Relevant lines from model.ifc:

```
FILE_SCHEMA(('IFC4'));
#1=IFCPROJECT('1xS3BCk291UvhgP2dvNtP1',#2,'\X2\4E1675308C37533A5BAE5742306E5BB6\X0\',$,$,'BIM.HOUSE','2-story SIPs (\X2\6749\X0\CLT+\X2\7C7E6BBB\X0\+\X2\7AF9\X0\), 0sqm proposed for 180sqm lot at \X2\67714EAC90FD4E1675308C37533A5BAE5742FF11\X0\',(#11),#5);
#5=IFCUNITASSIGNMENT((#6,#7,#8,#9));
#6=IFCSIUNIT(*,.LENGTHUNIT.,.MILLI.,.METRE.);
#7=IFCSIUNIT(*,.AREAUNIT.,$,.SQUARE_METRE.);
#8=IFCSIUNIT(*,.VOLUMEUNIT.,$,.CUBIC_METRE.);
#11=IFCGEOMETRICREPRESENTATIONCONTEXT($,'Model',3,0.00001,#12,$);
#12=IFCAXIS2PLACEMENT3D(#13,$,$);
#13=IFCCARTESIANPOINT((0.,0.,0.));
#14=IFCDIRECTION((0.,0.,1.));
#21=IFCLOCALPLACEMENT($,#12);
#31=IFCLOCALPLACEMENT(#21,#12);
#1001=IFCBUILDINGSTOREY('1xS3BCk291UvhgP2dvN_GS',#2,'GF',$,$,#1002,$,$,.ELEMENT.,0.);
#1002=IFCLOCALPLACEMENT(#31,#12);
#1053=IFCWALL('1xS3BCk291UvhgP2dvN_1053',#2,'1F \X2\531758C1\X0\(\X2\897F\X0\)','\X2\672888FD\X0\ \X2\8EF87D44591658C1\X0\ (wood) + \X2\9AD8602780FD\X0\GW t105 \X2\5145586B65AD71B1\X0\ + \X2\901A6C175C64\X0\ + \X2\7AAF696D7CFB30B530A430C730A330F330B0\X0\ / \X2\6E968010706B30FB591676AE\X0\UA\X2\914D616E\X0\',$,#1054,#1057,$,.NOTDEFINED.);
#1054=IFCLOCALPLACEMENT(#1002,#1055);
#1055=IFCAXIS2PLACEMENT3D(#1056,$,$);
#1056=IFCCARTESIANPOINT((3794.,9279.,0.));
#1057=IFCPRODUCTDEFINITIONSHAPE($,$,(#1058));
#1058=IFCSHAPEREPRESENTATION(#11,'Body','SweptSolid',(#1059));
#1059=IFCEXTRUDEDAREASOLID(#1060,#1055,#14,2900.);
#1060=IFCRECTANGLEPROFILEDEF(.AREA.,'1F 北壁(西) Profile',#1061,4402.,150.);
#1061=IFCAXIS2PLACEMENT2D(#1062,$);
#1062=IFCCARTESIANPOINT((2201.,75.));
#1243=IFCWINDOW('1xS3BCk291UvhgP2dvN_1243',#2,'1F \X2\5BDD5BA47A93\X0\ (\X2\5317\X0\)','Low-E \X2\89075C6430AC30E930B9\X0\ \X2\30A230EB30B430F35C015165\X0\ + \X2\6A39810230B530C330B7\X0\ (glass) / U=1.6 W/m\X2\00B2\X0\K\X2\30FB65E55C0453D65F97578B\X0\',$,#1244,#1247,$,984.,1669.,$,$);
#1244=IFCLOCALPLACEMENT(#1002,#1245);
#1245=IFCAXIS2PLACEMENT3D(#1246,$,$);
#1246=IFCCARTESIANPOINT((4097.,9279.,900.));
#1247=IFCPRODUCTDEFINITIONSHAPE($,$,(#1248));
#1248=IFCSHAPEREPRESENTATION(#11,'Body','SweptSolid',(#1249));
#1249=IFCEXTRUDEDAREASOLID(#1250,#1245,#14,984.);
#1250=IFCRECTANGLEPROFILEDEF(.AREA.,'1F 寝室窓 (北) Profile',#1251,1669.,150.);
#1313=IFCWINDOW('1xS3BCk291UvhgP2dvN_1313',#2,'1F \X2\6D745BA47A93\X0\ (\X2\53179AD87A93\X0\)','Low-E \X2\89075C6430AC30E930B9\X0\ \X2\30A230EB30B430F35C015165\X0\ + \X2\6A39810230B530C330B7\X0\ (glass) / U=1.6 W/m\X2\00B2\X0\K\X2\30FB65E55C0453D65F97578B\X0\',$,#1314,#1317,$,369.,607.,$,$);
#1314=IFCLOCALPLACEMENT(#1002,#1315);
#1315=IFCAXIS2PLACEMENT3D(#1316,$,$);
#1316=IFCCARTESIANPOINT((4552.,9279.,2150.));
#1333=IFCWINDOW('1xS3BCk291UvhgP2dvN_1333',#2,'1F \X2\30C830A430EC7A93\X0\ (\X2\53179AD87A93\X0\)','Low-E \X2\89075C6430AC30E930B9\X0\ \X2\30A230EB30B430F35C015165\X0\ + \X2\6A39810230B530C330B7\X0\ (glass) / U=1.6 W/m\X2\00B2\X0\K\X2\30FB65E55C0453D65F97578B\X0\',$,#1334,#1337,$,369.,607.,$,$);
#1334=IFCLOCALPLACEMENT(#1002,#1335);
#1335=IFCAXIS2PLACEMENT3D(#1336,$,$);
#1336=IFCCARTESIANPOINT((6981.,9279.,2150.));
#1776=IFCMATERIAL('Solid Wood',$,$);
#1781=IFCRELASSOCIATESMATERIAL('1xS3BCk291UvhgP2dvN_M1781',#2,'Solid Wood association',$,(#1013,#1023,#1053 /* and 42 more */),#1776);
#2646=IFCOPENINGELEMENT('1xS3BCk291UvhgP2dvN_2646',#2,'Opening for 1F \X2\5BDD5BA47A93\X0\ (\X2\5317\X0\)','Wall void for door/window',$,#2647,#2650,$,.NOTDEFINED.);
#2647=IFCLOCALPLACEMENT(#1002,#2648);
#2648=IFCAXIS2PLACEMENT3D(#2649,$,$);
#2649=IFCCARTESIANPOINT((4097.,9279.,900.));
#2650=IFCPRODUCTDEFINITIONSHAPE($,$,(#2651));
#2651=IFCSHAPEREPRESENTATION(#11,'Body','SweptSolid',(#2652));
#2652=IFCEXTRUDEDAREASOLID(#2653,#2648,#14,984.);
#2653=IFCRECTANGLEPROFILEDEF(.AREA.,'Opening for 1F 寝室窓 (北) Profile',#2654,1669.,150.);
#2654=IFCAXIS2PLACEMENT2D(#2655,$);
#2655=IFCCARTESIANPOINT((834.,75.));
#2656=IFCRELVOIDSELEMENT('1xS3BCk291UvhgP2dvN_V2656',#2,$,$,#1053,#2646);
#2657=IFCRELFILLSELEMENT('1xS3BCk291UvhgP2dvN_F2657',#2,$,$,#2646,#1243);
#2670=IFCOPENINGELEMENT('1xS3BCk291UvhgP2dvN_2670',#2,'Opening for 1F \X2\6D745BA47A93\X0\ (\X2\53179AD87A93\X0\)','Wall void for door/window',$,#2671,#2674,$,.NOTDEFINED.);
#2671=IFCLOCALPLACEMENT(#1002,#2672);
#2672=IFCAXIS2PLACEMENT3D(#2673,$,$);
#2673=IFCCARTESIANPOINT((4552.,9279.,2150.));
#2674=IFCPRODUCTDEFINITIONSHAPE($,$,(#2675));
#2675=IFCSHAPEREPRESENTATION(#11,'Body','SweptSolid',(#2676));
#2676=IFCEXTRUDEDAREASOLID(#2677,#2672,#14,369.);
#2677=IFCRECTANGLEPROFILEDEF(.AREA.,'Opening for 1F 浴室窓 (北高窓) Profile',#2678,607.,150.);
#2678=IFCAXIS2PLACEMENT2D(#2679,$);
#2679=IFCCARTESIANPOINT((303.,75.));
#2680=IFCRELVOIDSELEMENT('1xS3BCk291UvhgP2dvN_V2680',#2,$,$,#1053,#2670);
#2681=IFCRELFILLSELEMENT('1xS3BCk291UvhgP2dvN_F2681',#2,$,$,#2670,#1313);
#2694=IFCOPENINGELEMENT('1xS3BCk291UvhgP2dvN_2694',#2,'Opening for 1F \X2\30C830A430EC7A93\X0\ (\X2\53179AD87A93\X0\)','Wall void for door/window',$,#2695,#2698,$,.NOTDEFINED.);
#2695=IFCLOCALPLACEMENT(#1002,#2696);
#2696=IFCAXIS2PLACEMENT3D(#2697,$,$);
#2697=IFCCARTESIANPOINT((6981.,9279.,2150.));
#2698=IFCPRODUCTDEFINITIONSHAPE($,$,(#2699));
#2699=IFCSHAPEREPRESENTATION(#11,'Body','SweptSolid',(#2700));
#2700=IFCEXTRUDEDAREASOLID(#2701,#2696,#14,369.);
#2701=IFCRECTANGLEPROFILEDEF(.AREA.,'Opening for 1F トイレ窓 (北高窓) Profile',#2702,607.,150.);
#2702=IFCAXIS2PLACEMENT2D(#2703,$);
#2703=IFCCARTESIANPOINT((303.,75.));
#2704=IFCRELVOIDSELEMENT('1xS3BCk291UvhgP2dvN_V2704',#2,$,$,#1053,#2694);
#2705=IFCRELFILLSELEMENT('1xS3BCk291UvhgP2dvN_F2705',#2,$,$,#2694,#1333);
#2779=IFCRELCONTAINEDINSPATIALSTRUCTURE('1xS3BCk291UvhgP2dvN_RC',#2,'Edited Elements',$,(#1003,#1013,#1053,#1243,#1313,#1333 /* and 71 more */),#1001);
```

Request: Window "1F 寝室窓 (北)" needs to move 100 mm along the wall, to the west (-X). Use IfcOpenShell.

```python
import ifcopenshell
import ifcopenshell.api.geometry
import ifcopenshell.util.placement
import ifcopenshell.util.unit

model = ifcopenshell.open("model.ifc")
unit_scale = ifcopenshell.util.unit.calculate_unit_scale(model)

window = model.by_id(1243)
opening = window.FillsVoids[0].RelatingOpeningElement
wall = opening.VoidsElements[0].RelatingBuildingElement

wall_matrix = ifcopenshell.util.placement.get_local_placement(wall.ObjectPlacement)
shift = wall_matrix[:3, 0] * -0.1 / unit_scale
before = ifcopenshell.util.placement.get_local_placement(window.ObjectPlacement)[:3, 3].copy()

# The window is not placed relative to its opening, so move both.
for product in (opening, window):
    matrix = ifcopenshell.util.placement.get_local_placement(product.ObjectPlacement)
    matrix[:3, 3] += shift
    ifcopenshell.api.geometry.edit_object_placement(model, product=product, matrix=matrix, is_si=False)

after = ifcopenshell.util.placement.get_local_placement(window.ObjectPlacement)[:3, 3]
print("window moved by", (after - before).round(3) + 0.0)

model.write("model_updated.ifc")
```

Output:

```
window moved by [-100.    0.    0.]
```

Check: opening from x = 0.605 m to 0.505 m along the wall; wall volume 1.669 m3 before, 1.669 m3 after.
